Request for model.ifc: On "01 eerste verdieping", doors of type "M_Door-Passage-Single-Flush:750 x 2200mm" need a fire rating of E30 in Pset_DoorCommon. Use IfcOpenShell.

First a look at what the model holds.

```python
import ifcopenshell
import ifcopenshell.util.element

model = ifcopenshell.open("model.ifc")
print(model.schema)
storey = next(s for s in model.by_type("IfcBuildingStorey") if s.Name == "01 eerste verdieping")
doors = [e for e in ifcopenshell.util.element.get_decomposition(storey) if e.is_a("IfcDoor")]
seen = {}
for e in doors:
    element_type = ifcopenshell.util.element.get_type(e)
    key = (element_type.Name if element_type != e and element_type else None, ifcopenshell.util.element.get_pset(e, "Pset_DoorCommon", "FireRating"))
    seen[key] = seen.get(key, 0) + 1
for (name, value), count in sorted(seen.items(), key=str):
    print(count, "x", name, "|", value)
```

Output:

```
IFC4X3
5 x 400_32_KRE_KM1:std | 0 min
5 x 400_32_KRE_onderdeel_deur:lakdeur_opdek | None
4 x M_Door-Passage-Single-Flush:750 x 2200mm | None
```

```python
import ifcopenshell
import ifcopenshell.api.pset
import ifcopenshell.util.element

model = ifcopenshell.open("model.ifc")

storey = next(s for s in model.by_type("IfcBuildingStorey") if s.Name == "01 eerste verdieping")
doors = [e for e in ifcopenshell.util.element.get_decomposition(storey) if e.is_a("IfcDoor")]

count = 0
for e in doors:
    element_type = ifcopenshell.util.element.get_type(e)
    if element_type in (None, e) or element_type.Name != "M_Door-Passage-Single-Flush:750 x 2200mm":
        continue
    # add_pset returns the element's existing set when there is one.
    pset = ifcopenshell.api.pset.add_pset(model, product=e, name="Pset_DoorCommon")
    ifcopenshell.api.pset.edit_pset(model, pset=pset, properties={"FireRating": "E30"})
    count += 1

print(count, "doors updated")

model.write("model_rev.ifc")
```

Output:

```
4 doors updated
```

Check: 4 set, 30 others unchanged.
